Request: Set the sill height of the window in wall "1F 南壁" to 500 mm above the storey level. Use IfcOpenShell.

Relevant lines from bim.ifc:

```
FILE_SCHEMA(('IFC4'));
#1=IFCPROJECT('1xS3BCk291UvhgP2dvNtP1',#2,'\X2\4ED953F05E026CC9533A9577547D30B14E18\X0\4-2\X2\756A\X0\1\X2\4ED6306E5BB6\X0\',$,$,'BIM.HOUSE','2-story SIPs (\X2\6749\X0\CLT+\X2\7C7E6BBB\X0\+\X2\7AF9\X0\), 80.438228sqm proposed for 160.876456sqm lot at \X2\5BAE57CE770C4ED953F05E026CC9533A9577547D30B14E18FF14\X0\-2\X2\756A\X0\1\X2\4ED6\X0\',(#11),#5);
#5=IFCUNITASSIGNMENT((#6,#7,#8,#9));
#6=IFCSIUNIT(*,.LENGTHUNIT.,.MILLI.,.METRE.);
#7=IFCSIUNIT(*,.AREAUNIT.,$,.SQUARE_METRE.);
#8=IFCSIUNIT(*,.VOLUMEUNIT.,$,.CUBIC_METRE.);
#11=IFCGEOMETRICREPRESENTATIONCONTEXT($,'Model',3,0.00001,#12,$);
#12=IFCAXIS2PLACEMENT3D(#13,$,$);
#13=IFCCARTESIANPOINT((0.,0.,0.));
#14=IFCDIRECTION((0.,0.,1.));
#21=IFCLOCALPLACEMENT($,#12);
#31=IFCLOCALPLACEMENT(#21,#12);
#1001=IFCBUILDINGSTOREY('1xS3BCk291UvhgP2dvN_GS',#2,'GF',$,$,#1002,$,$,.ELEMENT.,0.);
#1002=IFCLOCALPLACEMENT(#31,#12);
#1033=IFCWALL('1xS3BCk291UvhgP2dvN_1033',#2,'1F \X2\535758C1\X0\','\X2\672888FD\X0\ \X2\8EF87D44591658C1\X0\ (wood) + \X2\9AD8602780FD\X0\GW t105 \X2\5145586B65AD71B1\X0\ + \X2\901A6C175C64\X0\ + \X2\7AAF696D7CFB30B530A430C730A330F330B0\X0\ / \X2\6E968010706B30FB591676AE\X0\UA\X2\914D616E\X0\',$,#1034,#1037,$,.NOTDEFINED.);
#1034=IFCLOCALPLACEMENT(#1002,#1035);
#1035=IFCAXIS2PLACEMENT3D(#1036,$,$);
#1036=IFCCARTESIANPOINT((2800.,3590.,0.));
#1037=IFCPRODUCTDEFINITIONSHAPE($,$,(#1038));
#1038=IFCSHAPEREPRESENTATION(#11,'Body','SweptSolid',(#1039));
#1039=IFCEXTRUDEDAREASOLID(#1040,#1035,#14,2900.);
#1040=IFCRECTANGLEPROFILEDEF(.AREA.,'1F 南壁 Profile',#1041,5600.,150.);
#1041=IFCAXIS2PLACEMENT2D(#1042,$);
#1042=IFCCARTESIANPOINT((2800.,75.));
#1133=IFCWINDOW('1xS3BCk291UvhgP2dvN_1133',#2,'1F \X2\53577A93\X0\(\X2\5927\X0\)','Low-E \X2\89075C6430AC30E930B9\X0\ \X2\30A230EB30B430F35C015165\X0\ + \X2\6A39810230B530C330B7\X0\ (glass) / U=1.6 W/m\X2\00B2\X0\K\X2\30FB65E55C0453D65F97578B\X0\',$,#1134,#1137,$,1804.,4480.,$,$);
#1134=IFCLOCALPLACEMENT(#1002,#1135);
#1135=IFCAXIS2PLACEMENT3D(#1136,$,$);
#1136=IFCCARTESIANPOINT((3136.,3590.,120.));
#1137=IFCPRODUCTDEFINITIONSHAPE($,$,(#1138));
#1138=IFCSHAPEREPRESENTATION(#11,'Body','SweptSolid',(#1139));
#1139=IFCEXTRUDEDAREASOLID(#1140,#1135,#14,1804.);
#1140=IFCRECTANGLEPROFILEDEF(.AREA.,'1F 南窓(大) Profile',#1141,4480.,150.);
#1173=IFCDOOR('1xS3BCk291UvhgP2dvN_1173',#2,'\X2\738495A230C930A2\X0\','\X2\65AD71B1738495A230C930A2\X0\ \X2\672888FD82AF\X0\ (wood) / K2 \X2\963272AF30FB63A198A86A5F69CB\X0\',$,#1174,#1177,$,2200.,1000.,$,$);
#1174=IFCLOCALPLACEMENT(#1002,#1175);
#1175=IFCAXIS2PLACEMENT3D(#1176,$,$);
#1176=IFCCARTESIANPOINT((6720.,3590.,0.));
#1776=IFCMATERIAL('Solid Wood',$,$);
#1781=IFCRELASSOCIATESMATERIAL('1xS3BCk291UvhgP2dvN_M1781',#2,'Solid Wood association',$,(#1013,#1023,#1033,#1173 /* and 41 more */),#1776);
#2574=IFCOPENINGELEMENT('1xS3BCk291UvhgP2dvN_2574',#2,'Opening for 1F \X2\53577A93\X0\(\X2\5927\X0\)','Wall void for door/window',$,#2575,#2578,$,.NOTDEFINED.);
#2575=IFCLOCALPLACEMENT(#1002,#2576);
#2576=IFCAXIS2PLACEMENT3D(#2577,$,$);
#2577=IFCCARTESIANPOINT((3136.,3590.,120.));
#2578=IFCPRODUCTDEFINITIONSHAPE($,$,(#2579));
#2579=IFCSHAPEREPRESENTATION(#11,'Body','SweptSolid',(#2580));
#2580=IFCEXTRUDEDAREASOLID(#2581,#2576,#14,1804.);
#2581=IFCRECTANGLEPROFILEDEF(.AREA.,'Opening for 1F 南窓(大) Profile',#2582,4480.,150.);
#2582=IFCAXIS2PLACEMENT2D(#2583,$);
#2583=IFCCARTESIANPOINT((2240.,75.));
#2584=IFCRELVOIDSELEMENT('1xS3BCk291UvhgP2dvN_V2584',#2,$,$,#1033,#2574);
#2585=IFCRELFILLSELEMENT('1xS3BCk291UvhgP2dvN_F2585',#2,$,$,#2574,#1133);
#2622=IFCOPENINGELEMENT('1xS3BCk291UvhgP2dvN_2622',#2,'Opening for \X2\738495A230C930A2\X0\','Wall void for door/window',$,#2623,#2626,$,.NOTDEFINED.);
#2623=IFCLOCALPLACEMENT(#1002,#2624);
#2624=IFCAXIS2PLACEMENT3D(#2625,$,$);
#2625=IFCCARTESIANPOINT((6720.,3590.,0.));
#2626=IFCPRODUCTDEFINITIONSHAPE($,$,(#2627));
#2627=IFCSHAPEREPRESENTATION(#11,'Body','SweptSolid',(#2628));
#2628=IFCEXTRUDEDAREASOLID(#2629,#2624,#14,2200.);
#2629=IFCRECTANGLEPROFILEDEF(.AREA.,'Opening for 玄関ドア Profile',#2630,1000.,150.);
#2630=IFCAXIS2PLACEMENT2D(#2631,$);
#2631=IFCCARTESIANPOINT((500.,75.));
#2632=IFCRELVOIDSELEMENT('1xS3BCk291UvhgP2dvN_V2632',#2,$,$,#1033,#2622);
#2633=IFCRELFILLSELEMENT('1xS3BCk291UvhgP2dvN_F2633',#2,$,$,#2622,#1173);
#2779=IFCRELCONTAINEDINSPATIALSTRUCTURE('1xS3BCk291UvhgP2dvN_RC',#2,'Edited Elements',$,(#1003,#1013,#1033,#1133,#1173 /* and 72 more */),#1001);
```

```python
import numpy as np
import ifcopenshell
import ifcopenshell.api.geometry
import ifcopenshell.geom
import ifcopenshell.util.element
import ifcopenshell.util.placement
import ifcopenshell.util.shape
import ifcopenshell.util.unit

model = ifcopenshell.open("bim.ifc")
unit_scale = ifcopenshell.util.unit.calculate_unit_scale(model)

window = model.by_id(1133)
opening = window.FillsVoids[0].RelatingOpeningElement
storey = ifcopenshell.util.element.get_container(window, ifc_class="IfcBuildingStorey")
level = ifcopenshell.util.placement.get_local_placement(storey.ObjectPlacement)[2, 3]

# The opening's origin need not be at the sill, so measure its lowest point.
shape = ifcopenshell.geom.create_shape(ifcopenshell.geom.settings(), opening)
bottom = ifcopenshell.util.shape.get_shape_bottom_elevation(shape, shape.geometry) / unit_scale
dz = level + 500.0 - bottom

shift = np.array([0.0, 0.0, dz])
# The window is not placed relative to its opening, so move both.
for product in (opening, window):
    matrix = ifcopenshell.util.placement.get_local_placement(product.ObjectPlacement)
    matrix[:3, 3] += shift
    ifcopenshell.api.geometry.edit_object_placement(model, product=product, matrix=matrix, is_si=False)

print(f"moved by {dz * unit_scale:+.3f} m")

model.write("bim-out.ifc")
```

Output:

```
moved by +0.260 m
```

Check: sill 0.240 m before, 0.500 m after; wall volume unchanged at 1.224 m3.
